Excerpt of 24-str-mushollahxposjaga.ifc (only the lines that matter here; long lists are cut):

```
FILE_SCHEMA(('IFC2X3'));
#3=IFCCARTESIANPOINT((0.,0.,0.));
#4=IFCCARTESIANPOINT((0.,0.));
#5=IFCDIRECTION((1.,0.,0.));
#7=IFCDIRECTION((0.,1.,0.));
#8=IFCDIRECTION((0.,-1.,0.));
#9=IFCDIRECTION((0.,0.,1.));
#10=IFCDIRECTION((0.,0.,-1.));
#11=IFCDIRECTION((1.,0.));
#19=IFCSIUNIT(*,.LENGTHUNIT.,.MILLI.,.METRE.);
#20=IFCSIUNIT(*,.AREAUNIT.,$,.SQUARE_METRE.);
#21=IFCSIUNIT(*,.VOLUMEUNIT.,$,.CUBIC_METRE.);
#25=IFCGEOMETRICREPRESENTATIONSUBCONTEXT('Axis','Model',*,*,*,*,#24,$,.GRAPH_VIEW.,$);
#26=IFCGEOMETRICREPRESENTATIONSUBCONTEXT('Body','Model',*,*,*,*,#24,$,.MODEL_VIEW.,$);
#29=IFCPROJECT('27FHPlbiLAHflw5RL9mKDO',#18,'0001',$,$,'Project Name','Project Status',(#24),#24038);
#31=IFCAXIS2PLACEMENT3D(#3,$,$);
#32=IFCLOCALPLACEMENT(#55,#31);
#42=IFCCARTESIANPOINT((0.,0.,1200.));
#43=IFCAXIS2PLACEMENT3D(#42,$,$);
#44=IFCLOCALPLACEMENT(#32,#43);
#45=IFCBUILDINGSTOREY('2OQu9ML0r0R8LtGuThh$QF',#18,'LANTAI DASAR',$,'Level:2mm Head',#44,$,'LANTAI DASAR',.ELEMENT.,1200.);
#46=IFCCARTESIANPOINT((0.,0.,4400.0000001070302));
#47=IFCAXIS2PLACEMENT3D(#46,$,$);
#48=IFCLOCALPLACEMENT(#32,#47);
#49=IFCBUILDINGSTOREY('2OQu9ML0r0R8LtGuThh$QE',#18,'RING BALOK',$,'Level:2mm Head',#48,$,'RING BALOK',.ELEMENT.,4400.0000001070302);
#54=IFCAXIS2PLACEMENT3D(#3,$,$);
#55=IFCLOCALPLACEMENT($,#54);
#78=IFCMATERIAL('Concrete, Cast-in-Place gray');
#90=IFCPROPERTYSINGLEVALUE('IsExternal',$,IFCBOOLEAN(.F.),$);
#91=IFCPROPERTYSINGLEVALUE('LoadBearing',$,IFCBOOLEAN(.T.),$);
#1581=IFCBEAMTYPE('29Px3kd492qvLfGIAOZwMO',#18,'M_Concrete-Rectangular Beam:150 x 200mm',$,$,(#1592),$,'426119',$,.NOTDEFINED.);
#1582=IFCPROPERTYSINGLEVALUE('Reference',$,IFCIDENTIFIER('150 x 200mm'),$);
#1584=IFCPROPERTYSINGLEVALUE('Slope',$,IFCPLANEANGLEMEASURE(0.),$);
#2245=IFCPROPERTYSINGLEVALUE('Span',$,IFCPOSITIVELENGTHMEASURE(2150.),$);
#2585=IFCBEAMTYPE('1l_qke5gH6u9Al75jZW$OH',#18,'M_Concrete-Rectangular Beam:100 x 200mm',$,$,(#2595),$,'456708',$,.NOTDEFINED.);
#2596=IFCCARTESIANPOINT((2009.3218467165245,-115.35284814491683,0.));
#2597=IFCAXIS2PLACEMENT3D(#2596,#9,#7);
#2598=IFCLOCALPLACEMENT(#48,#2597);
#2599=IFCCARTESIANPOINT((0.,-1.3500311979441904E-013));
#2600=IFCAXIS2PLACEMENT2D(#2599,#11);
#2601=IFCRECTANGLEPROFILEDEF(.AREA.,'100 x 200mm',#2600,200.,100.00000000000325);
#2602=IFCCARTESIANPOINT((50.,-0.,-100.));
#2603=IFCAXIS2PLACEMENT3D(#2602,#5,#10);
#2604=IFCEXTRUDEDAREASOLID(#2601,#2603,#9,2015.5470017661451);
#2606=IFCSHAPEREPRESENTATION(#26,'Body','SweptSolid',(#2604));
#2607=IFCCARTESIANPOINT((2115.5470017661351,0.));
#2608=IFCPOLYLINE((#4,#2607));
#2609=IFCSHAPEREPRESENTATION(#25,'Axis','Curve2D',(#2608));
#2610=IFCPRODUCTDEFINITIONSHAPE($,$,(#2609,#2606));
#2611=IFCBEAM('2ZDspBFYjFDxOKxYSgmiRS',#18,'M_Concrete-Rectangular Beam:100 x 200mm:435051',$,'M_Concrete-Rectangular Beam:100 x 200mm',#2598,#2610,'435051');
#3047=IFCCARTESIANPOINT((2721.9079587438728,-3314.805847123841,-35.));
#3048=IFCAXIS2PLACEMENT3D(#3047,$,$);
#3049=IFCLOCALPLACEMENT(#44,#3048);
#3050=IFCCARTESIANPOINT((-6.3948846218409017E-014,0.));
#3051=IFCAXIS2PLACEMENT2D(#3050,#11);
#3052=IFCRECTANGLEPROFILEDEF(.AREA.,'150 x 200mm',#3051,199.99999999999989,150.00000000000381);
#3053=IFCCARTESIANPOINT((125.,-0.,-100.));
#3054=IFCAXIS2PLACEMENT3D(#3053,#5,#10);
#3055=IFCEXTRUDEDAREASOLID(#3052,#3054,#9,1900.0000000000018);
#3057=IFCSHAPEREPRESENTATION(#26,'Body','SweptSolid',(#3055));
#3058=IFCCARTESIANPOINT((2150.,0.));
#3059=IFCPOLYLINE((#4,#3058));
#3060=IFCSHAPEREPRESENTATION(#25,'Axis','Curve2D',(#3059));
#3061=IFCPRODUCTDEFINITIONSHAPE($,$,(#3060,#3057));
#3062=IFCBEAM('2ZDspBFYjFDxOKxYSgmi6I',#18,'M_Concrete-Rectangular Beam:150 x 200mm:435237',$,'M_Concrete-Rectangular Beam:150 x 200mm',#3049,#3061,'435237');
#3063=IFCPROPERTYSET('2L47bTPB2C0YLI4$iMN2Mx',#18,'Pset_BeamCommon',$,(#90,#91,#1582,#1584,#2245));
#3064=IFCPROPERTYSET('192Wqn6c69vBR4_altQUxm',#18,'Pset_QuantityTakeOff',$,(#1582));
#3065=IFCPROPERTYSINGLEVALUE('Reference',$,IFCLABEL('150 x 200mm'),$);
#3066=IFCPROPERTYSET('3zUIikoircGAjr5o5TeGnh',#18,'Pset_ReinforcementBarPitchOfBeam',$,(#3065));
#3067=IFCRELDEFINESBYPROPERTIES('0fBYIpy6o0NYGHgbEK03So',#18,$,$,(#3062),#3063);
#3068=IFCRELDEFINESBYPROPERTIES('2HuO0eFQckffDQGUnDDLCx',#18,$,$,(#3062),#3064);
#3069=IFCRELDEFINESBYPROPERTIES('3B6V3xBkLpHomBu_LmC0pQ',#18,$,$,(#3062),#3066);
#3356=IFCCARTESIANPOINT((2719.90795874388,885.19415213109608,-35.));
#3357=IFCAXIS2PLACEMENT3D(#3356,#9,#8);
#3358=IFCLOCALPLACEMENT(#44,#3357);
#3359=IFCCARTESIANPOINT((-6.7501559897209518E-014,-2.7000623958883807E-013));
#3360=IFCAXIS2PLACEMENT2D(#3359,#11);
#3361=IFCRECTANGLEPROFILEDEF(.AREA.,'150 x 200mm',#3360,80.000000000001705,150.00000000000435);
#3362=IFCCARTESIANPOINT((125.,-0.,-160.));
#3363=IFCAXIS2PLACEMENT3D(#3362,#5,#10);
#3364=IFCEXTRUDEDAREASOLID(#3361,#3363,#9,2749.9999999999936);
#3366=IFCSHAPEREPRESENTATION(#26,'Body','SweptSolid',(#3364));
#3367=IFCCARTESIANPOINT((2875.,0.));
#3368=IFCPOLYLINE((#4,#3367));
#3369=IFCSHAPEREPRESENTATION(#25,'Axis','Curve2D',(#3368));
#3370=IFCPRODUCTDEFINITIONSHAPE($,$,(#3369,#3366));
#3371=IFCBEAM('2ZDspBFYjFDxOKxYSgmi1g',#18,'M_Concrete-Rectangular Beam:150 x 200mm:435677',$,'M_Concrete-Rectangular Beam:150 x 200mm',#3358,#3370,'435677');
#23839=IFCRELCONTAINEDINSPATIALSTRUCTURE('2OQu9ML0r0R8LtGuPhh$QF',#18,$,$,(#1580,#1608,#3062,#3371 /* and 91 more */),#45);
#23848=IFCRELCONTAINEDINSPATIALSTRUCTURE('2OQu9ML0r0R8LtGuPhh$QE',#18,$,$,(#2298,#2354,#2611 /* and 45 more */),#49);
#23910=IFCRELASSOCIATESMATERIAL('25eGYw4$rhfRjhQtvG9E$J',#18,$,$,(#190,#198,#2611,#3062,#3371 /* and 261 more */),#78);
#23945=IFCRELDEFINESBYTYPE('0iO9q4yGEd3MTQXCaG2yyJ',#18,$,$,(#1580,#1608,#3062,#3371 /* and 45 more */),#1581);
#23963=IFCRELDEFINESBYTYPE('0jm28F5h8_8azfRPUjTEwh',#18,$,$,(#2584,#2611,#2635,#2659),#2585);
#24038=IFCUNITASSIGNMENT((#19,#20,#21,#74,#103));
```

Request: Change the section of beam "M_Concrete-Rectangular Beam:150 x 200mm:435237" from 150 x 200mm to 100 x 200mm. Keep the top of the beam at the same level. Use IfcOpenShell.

```python
import ifcopenshell
import ifcopenshell.api.pset
import ifcopenshell.api.type
import ifcopenshell.util.element
import ifcopenshell.util.representation

model = ifcopenshell.open("24-str-mushollahxposjaga.ifc")

member = model.by_guid("2ZDspBFYjFDxOKxYSgmi6I")
source = next(p for p in model.by_type("IfcRectangleProfileDef") if p.ProfileName == "100 x 200mm")

body = ifcopenshell.util.representation.get_representation(member, "Model", "Body")
solid = body.Items[0]
old_profile = solid.SweptArea

# Copy the section's sizes but keep this member's own profile position.
profile = ifcopenshell.util.element.copy(model, source)
# Profiles are centred, so shift by half the change in depth to hold the top.
shift = (old_profile.XDim - profile.XDim) / 2
x, y = old_profile.Position.Location.Coordinates
up = (-1.0, 0.0)  # upwards, in the solid's own plane
location = model.createIfcCartesianPoint((x + up[0] * shift, y + up[1] * shift))
profile.Position = model.createIfcAxis2Placement2D(location, old_profile.Position.RefDirection)
solid.SweptArea = profile
if not model.get_total_inverses(old_profile):
    ifcopenshell.util.element.remove_deep2(model, old_profile)

new_type = model.by_guid("1l_qke5gH6u9Al75jZW$OH")
ifcopenshell.api.type.assign_type(
    model, related_objects=[member], relating_type=new_type, should_map_representations=False
)
member.Name = member.Name.replace("150 x 200mm", "100 x 200mm")
member.ObjectType = "M_Concrete-Rectangular Beam:100 x 200mm"
pset = model.by_id(ifcopenshell.util.element.get_pset(member, "Pset_BeamCommon", should_inherit=False)["id"])
ifcopenshell.api.pset.edit_pset(model, pset=pset, properties={"Reference": "100 x 200mm"})
pset = model.by_id(ifcopenshell.util.element.get_pset(member, "Pset_QuantityTakeOff", should_inherit=False)["id"])
ifcopenshell.api.pset.edit_pset(model, pset=pset, properties={"Reference": "100 x 200mm"})
pset = model.by_id(ifcopenshell.util.element.get_pset(member, "Pset_ReinforcementBarPitchOfBeam", should_inherit=False)["id"])
ifcopenshell.api.pset.edit_pset(model, pset=pset, properties={"Reference": "100 x 200mm"})

print(solid.SweptArea)

model.write("24-str-mushollahxposjaga-out.ifc")
```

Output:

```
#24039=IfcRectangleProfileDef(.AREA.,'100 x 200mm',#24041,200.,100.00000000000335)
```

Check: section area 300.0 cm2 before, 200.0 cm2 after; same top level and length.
